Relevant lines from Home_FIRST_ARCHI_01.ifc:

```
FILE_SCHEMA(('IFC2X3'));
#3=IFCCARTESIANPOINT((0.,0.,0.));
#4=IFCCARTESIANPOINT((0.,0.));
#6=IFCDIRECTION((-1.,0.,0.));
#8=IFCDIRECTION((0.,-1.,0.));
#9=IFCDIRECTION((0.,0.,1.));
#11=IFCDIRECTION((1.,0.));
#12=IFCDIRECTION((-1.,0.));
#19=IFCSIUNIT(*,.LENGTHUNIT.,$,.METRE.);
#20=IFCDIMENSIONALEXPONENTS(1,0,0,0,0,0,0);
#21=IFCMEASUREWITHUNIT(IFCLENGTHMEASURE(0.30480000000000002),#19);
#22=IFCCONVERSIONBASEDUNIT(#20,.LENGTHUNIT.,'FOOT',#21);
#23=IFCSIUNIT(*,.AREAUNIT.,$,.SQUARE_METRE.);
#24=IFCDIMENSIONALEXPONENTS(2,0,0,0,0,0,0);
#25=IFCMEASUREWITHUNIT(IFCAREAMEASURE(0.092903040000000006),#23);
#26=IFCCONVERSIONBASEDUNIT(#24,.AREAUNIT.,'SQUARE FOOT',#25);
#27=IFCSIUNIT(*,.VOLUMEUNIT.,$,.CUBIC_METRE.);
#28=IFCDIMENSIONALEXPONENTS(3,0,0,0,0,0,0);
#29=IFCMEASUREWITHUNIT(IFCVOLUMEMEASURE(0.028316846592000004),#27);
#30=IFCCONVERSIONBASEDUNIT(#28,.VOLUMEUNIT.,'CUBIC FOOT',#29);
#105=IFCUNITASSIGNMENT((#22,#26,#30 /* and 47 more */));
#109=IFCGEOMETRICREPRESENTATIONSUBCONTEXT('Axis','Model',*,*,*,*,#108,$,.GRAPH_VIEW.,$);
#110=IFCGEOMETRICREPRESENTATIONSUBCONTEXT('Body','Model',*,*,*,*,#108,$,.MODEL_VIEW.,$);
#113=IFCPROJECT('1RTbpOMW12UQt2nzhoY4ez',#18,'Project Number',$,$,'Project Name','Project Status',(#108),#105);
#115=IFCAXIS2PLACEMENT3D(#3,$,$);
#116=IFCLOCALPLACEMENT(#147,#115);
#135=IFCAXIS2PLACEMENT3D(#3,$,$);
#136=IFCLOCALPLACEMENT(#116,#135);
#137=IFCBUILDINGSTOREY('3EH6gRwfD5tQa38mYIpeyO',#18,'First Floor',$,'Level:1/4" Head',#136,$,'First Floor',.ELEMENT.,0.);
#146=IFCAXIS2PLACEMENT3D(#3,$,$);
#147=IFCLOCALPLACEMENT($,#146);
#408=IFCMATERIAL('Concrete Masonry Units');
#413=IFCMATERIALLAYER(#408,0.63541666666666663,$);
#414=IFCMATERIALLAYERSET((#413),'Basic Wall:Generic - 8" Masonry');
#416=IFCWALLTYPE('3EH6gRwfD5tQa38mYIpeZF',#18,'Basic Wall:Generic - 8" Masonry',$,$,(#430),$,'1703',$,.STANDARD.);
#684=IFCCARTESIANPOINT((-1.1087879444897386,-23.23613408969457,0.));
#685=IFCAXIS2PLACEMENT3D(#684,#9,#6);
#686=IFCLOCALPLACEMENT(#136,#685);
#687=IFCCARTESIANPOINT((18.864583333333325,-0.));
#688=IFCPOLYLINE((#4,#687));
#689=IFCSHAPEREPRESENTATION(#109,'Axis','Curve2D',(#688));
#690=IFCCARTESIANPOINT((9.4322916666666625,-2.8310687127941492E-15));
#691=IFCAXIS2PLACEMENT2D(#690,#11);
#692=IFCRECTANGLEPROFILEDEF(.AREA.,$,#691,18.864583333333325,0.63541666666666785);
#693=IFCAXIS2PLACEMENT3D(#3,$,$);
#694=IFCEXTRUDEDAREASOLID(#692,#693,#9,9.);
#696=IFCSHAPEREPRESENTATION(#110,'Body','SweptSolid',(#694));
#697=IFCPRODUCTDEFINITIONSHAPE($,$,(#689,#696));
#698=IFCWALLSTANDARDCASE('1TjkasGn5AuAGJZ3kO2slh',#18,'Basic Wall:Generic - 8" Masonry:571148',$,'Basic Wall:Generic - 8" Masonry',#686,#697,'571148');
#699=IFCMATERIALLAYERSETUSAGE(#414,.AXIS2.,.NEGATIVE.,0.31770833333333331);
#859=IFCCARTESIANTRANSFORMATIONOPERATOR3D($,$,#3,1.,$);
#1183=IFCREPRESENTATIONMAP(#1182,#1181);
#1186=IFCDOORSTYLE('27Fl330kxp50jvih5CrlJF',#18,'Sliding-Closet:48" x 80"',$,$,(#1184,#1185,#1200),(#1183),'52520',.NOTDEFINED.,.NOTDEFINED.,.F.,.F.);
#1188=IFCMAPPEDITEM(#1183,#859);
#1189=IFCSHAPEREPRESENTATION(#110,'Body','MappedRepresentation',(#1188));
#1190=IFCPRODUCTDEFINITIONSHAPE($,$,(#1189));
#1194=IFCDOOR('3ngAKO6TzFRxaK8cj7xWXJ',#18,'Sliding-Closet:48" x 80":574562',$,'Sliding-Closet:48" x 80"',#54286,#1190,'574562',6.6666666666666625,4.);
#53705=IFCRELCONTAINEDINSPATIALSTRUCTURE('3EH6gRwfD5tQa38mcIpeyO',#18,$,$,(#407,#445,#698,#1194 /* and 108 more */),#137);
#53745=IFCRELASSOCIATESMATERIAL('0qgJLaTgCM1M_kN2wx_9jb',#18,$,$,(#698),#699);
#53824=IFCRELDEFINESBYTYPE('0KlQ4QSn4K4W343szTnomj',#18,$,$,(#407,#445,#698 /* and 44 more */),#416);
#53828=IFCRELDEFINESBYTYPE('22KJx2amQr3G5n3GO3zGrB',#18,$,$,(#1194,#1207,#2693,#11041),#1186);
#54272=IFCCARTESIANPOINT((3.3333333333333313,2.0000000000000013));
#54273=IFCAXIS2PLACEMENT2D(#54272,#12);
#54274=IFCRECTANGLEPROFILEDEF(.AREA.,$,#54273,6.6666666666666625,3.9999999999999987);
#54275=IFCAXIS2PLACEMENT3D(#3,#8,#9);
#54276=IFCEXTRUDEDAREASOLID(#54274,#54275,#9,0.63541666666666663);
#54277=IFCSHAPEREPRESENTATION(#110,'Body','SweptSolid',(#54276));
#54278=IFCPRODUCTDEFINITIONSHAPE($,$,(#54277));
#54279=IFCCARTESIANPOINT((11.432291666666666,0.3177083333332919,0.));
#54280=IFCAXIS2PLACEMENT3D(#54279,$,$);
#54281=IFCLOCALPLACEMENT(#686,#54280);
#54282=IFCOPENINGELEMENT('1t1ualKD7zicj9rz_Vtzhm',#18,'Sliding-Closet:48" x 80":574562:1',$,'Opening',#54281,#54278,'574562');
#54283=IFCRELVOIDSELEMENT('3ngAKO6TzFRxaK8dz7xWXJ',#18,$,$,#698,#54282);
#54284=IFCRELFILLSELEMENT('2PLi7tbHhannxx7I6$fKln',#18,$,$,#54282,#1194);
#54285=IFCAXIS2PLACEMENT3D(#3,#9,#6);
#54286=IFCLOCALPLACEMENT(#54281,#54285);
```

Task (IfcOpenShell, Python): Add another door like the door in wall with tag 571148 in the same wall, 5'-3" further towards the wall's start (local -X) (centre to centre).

```python
import ifcopenshell
import ifcopenshell.api.feature
import ifcopenshell.api.geometry
import ifcopenshell.api.root
import ifcopenshell.geom
import ifcopenshell.util.element
import ifcopenshell.util.placement
import ifcopenshell.util.shape
import ifcopenshell.util.unit

model = ifcopenshell.open("Home_FIRST_ARCHI_01.ifc")
unit_scale = ifcopenshell.util.unit.calculate_unit_scale(model)
settings = ifcopenshell.geom.settings()


def volume(element):
    """Net volume in cubic metres, openings subtracted."""
    shape = ifcopenshell.geom.create_shape(settings, element)
    return ifcopenshell.util.shape.get_volume(shape.geometry)


def reuse_history(source, copy):
    """copy_class also copies each property set's owner history, people and application; keep the originals."""
    for rel in copy.IsDefinedBy:
        if rel.is_a("IfcRelDefinesByProperties") and (history := rel.RelatingPropertyDefinition.OwnerHistory):
            rel.RelatingPropertyDefinition.OwnerHistory = source.OwnerHistory
            ifcopenshell.util.element.remove_deep2(model, history)


door = model.by_guid("3ngAKO6TzFRxaK8cj7xWXJ")
opening = door.FillsVoids[0].RelatingOpeningElement
wall = opening.VoidsElements[0].RelatingBuildingElement
before = volume(wall)
shift = ifcopenshell.util.placement.get_local_placement(wall.ObjectPlacement)[:3, 0] * -63 * 0.0254 / unit_scale

# copy_class copies the void relationship, type, container and properties, but no geometry.
new_opening = ifcopenshell.api.root.copy_class(model, product=opening)
new_opening.Representation = ifcopenshell.util.element.copy_deep(
    model, opening.Representation, exclude=["IfcGeometricRepresentationContext", "IfcRepresentationMap"]
)
new_opening.Name = 'Sliding-Closet:48" x 80"'
new_opening.Tag = None
new_door = ifcopenshell.api.root.copy_class(model, product=door)
new_door.Representation = ifcopenshell.util.element.copy_deep(
    model, door.Representation, exclude=["IfcGeometricRepresentationContext", "IfcRepresentationMap"]
)
new_door.Name = 'Sliding-Closet:48" x 80"'
new_door.Tag = None
reuse_history(door, new_door)
fills = ifcopenshell.api.feature.add_filling(model, opening=new_opening, element=new_door)
fills.OwnerHistory = new_door.OwnerHistory  # required in IFC2X3

for old, new in ((opening, new_opening), (door, new_door)):
    matrix = ifcopenshell.util.placement.get_local_placement(old.ObjectPlacement)
    matrix[:3, 3] += shift
    ifcopenshell.api.geometry.edit_object_placement(model, product=new, matrix=matrix, is_si=False)

after = volume(wall)

print(f"wall volume {before:.3f} -> {after:.3f} m3")

model.write("Home_FIRST_ARCHI_01_v2.ifc")
```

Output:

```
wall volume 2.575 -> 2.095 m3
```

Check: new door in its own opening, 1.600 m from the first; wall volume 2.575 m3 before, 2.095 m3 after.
